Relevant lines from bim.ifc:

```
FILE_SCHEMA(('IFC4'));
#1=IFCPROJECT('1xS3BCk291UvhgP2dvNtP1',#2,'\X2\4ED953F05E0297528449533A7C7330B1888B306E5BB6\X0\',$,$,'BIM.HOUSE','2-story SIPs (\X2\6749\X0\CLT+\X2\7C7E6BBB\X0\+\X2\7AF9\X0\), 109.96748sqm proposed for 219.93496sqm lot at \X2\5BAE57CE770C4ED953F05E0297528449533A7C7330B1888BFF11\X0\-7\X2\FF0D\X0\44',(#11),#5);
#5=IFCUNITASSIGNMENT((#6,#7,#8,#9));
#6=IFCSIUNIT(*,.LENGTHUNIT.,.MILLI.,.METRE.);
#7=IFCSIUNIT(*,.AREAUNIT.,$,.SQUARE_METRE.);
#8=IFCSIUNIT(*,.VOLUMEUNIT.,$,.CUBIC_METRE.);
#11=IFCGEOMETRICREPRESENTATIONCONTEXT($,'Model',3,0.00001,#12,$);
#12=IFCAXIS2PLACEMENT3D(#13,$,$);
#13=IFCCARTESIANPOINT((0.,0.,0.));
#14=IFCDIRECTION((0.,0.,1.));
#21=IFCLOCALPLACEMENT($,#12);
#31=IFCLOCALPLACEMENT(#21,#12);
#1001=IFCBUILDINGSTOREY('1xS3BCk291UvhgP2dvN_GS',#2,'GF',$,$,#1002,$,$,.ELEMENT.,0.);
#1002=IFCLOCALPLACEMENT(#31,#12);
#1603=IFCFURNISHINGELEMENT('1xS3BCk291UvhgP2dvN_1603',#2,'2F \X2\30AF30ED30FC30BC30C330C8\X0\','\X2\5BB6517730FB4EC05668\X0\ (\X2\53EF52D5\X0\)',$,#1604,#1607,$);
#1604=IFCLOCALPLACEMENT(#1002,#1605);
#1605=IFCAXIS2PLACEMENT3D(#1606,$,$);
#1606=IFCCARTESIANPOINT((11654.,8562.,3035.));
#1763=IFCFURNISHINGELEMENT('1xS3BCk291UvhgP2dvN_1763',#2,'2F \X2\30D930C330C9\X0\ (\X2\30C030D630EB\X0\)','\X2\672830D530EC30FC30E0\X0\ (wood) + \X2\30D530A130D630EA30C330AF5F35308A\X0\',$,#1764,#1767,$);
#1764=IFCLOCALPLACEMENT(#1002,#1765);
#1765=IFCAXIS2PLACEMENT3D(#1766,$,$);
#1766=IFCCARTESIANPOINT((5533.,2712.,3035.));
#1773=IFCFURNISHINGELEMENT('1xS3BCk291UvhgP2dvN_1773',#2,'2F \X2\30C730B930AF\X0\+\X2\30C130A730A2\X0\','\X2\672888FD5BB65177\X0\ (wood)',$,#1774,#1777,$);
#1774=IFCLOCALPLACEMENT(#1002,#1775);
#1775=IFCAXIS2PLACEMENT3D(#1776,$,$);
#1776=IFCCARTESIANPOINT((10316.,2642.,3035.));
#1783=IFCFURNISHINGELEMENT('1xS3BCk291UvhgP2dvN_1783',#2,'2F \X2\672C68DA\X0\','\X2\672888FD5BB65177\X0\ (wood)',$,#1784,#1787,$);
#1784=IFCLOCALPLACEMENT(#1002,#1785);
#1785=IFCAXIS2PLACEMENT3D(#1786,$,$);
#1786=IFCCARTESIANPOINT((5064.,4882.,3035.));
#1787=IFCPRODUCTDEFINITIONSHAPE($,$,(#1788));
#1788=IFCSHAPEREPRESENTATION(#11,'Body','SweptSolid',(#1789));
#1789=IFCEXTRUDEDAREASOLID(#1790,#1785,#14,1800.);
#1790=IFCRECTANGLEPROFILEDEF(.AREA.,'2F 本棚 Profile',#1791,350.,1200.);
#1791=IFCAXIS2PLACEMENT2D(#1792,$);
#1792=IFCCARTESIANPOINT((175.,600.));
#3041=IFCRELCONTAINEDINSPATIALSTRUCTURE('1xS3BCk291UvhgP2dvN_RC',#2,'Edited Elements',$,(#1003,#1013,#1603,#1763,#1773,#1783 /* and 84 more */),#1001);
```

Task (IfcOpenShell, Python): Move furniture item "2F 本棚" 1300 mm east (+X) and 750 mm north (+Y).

```python
import ifcopenshell
import ifcopenshell.api.geometry
import ifcopenshell.util.placement
import ifcopenshell.util.unit

model = ifcopenshell.open("bim.ifc")
unit_scale = ifcopenshell.util.unit.calculate_unit_scale(model)

item = model.by_guid("1xS3BCk291UvhgP2dvN_1783")
matrix = ifcopenshell.util.placement.get_local_placement(item.ObjectPlacement)
matrix[0, 3] += 1.3 / unit_scale
matrix[1, 3] += 0.75 / unit_scale
ifcopenshell.api.geometry.edit_object_placement(model, product=item, matrix=matrix, is_si=False)

print(ifcopenshell.util.placement.get_local_placement(item.ObjectPlacement).round(3) + 0.0)

model.write("bim_v2.ifc")
```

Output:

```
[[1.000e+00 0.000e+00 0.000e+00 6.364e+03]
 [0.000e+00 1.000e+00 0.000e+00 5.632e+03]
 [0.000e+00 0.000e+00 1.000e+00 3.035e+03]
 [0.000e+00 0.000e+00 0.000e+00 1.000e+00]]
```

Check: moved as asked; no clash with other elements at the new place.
